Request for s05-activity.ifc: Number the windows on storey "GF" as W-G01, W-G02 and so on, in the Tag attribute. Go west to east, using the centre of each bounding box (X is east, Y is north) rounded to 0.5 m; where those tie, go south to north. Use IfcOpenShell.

First a look at what the model holds.

```python
import ifcopenshell
import ifcopenshell.util.element
import ifcopenshell.util.placement

model = ifcopenshell.open("s05-activity.ifc")
print(model.schema)
storey = next(s for s in model.by_type("IfcBuildingStorey") if s.Name == "GF")
windows = [e for e in ifcopenshell.util.element.get_decomposition(storey) if e.is_a("IfcWindow")]
for e in sorted(windows, key=lambda e: e.id()):
    origin = ifcopenshell.util.placement.get_local_placement(e.ObjectPlacement)[:3, 3]
    print(e.id(), e.Tag, e.Name, origin.round(2) + 0.0, sep=" | ")
```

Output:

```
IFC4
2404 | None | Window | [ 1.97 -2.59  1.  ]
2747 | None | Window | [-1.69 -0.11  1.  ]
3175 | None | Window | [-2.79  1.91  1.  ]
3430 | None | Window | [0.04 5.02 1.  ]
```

```python
import ifcopenshell
import ifcopenshell.geom
import ifcopenshell.util.element
import ifcopenshell.util.shape

model = ifcopenshell.open("s05-activity.ifc")
settings = ifcopenshell.geom.settings()
settings.set("use-world-coords", True)


def centre(element):
    shape = ifcopenshell.geom.create_shape(settings, element)
    return ifcopenshell.util.shape.get_bbox_centroid(shape.geometry)


storey = next(s for s in model.by_type("IfcBuildingStorey") if s.Name == "GF")
windows = [e for e in ifcopenshell.util.element.get_decomposition(storey) if e.is_a("IfcWindow")]

# Insertion points can sit at a corner or the storey origin, so sort by the geometry (in metres).
centres = {e: centre(e) for e in windows}
windows.sort(key=lambda e: (round(centres[e][0] / 0.5), centres[e][1]))

for i, e in enumerate(windows, start=1):
    number = f"W-G{i:02d}"
    e.Tag = number
    print(e.id(), number)

model.write("s05-activity_edited.ifc")
```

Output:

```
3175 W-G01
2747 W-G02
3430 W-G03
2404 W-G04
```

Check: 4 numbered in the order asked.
